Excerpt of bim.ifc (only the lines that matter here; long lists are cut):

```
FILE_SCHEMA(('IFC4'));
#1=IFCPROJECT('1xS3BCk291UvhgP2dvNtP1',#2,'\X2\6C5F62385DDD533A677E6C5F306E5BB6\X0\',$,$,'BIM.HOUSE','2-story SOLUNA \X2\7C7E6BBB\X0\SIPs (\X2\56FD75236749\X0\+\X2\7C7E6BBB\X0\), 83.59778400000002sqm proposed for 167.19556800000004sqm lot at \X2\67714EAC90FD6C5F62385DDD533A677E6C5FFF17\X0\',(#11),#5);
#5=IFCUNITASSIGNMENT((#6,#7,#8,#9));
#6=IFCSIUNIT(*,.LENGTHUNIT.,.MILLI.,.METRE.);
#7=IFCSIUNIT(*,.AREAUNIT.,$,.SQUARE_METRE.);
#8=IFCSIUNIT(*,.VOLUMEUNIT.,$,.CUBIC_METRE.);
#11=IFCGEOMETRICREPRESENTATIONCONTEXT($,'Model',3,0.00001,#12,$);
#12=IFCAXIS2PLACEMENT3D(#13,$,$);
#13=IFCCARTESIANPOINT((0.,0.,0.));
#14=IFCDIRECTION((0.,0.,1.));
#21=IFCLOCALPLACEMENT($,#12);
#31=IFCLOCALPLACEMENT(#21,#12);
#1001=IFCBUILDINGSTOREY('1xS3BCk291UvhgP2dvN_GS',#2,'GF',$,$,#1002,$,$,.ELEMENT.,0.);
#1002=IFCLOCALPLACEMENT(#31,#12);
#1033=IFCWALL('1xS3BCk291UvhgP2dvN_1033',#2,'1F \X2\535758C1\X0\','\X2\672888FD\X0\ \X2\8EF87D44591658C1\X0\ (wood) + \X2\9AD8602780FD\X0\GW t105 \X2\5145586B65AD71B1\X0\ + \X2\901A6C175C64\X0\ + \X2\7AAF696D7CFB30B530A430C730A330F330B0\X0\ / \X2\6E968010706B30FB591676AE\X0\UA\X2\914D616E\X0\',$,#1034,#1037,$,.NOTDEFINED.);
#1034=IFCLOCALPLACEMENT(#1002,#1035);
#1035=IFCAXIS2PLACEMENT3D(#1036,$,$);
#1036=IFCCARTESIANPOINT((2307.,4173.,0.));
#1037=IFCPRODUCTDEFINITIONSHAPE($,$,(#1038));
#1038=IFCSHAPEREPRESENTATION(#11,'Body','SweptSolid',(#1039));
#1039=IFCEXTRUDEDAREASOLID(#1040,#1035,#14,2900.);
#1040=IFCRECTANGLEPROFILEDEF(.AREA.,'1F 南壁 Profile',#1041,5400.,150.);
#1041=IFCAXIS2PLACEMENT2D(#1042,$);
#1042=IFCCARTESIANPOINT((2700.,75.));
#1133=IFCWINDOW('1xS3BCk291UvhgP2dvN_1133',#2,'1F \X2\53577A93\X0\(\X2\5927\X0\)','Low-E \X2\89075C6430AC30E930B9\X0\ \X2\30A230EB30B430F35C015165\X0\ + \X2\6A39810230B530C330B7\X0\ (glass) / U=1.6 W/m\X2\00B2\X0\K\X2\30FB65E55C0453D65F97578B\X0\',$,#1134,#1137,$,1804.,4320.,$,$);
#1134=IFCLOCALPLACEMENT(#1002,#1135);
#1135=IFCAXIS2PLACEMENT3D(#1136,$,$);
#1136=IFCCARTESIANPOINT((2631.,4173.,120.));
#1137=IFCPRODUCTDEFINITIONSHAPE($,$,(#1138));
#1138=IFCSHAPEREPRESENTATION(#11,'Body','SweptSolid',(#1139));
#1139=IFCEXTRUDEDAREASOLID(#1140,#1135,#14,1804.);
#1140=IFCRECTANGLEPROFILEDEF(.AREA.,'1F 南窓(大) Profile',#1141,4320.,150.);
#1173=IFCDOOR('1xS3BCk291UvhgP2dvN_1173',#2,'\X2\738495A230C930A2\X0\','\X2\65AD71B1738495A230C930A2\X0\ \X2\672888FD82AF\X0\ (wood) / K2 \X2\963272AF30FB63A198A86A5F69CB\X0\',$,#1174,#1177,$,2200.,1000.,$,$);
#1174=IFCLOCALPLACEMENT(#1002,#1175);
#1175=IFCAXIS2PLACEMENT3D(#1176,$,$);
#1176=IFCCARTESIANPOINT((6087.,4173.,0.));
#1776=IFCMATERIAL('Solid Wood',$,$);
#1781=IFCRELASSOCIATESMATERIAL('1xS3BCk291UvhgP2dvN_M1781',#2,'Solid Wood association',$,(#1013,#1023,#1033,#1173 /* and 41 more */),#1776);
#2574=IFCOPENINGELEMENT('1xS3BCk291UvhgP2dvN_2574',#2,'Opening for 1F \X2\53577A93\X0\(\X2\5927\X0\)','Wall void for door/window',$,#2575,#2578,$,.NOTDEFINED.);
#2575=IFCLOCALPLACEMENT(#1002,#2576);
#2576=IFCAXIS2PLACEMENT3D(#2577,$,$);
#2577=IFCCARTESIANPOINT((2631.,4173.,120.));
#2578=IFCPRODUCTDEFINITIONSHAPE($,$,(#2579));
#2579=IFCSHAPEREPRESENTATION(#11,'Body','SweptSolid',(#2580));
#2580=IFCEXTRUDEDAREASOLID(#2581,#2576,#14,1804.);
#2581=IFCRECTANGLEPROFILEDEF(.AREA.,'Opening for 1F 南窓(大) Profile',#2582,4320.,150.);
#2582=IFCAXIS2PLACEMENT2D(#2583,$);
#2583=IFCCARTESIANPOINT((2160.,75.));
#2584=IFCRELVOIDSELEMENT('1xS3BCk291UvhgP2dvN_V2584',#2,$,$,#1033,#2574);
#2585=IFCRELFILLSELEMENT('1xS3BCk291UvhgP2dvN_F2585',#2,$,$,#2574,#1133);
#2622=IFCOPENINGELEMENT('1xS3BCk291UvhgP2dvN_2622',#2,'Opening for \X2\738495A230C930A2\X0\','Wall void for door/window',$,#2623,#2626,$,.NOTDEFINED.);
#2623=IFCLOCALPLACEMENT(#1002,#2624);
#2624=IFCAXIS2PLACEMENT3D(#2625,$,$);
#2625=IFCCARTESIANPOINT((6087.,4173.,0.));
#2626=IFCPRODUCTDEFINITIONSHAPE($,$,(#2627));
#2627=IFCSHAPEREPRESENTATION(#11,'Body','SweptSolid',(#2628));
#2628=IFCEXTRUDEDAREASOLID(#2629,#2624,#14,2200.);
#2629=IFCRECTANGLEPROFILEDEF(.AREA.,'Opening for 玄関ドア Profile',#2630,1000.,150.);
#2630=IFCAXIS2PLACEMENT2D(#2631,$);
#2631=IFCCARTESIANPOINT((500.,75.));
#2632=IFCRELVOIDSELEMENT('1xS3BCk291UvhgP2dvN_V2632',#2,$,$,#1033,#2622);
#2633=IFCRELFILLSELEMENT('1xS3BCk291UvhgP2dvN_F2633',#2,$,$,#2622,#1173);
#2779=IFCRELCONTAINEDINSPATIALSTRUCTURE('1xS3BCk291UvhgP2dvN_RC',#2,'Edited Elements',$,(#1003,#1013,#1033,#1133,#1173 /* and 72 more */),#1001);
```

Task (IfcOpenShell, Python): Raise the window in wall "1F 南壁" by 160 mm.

```python
import numpy as np
import ifcopenshell
import ifcopenshell.api.geometry
import ifcopenshell.util.placement
import ifcopenshell.util.unit

model = ifcopenshell.open("bim.ifc")
unit_scale = ifcopenshell.util.unit.calculate_unit_scale(model)

window = model.by_guid("1xS3BCk291UvhgP2dvN_1133")
opening = window.FillsVoids[0].RelatingOpeningElement
dz = 0.16 / unit_scale

shift = np.array([0.0, 0.0, dz])
# The window is not placed relative to its opening, so move both.
for product in (opening, window):
    matrix = ifcopenshell.util.placement.get_local_placement(product.ObjectPlacement)
    matrix[:3, 3] += shift
    ifcopenshell.api.geometry.edit_object_placement(model, product=product, matrix=matrix, is_si=False)

print(f"moved by {dz * unit_scale:+.3f} m")

model.write("bim-out.ifc")
```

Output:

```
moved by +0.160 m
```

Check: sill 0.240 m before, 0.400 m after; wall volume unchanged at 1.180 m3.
